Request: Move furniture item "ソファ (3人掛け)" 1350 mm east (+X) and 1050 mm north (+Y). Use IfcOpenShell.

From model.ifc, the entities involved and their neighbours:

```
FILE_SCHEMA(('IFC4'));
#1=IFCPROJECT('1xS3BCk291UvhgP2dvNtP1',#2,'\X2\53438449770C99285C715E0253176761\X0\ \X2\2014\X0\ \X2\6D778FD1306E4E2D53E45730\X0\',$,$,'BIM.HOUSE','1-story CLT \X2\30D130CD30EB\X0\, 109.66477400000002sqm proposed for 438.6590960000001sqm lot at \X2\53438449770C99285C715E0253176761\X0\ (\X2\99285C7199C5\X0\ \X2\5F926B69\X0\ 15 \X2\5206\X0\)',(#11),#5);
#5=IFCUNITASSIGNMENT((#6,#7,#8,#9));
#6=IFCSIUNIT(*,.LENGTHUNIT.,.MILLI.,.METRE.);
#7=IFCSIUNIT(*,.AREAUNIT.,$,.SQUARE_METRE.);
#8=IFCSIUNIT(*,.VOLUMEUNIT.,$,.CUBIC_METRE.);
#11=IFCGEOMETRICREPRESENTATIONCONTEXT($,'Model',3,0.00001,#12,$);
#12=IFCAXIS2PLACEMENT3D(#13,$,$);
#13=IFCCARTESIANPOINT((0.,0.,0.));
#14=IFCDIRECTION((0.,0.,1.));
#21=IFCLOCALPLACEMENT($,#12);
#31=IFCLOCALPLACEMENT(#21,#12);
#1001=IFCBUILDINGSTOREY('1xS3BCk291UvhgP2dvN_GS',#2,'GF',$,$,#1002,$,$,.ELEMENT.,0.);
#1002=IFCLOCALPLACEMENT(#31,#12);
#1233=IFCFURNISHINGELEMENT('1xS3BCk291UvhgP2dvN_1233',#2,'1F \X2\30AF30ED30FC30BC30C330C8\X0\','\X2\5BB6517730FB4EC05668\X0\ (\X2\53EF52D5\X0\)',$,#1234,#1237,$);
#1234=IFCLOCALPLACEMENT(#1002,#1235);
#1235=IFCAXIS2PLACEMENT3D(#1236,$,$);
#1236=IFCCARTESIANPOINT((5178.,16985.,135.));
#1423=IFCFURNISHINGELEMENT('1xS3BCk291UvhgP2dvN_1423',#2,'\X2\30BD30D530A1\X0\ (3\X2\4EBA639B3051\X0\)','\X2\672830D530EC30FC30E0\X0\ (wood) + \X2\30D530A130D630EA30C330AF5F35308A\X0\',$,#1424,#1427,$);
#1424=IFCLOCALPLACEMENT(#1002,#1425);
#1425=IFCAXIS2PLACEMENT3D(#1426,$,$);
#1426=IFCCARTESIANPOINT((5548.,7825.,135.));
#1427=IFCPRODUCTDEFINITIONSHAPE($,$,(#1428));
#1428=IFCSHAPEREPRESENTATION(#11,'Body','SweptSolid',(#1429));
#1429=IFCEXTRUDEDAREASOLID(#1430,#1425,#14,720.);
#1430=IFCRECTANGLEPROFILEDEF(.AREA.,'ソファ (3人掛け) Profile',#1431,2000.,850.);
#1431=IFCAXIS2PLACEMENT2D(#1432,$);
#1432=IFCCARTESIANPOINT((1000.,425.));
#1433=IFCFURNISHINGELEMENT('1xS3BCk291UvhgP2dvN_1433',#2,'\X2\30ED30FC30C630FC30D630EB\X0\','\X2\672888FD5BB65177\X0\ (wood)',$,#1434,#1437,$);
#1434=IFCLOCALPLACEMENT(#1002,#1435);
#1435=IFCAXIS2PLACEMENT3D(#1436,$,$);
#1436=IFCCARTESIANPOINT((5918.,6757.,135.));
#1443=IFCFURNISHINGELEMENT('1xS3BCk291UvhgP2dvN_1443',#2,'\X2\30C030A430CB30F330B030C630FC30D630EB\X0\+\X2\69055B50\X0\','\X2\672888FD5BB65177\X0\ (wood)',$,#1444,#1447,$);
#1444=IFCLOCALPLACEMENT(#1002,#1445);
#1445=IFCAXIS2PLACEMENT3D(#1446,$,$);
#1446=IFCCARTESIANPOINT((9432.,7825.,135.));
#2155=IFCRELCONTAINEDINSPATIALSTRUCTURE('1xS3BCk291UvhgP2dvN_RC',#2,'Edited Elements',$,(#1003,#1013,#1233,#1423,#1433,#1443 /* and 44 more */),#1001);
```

```python
import ifcopenshell
import ifcopenshell.api.geometry
import ifcopenshell.util.placement

model = ifcopenshell.open("model.ifc")

item = model.by_guid("1xS3BCk291UvhgP2dvN_1423")
matrix = ifcopenshell.util.placement.get_local_placement(item.ObjectPlacement)
matrix[0, 3] += 1350.0
matrix[1, 3] += 1050.0
ifcopenshell.api.geometry.edit_object_placement(model, product=item, matrix=matrix, is_si=False)

print(ifcopenshell.util.placement.get_local_placement(item.ObjectPlacement).round(3) + 0.0)

model.write("model-out.ifc")
```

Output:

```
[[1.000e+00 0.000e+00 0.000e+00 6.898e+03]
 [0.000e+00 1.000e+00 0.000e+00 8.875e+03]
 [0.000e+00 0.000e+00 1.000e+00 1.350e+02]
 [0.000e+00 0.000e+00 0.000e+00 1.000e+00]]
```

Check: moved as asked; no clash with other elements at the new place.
